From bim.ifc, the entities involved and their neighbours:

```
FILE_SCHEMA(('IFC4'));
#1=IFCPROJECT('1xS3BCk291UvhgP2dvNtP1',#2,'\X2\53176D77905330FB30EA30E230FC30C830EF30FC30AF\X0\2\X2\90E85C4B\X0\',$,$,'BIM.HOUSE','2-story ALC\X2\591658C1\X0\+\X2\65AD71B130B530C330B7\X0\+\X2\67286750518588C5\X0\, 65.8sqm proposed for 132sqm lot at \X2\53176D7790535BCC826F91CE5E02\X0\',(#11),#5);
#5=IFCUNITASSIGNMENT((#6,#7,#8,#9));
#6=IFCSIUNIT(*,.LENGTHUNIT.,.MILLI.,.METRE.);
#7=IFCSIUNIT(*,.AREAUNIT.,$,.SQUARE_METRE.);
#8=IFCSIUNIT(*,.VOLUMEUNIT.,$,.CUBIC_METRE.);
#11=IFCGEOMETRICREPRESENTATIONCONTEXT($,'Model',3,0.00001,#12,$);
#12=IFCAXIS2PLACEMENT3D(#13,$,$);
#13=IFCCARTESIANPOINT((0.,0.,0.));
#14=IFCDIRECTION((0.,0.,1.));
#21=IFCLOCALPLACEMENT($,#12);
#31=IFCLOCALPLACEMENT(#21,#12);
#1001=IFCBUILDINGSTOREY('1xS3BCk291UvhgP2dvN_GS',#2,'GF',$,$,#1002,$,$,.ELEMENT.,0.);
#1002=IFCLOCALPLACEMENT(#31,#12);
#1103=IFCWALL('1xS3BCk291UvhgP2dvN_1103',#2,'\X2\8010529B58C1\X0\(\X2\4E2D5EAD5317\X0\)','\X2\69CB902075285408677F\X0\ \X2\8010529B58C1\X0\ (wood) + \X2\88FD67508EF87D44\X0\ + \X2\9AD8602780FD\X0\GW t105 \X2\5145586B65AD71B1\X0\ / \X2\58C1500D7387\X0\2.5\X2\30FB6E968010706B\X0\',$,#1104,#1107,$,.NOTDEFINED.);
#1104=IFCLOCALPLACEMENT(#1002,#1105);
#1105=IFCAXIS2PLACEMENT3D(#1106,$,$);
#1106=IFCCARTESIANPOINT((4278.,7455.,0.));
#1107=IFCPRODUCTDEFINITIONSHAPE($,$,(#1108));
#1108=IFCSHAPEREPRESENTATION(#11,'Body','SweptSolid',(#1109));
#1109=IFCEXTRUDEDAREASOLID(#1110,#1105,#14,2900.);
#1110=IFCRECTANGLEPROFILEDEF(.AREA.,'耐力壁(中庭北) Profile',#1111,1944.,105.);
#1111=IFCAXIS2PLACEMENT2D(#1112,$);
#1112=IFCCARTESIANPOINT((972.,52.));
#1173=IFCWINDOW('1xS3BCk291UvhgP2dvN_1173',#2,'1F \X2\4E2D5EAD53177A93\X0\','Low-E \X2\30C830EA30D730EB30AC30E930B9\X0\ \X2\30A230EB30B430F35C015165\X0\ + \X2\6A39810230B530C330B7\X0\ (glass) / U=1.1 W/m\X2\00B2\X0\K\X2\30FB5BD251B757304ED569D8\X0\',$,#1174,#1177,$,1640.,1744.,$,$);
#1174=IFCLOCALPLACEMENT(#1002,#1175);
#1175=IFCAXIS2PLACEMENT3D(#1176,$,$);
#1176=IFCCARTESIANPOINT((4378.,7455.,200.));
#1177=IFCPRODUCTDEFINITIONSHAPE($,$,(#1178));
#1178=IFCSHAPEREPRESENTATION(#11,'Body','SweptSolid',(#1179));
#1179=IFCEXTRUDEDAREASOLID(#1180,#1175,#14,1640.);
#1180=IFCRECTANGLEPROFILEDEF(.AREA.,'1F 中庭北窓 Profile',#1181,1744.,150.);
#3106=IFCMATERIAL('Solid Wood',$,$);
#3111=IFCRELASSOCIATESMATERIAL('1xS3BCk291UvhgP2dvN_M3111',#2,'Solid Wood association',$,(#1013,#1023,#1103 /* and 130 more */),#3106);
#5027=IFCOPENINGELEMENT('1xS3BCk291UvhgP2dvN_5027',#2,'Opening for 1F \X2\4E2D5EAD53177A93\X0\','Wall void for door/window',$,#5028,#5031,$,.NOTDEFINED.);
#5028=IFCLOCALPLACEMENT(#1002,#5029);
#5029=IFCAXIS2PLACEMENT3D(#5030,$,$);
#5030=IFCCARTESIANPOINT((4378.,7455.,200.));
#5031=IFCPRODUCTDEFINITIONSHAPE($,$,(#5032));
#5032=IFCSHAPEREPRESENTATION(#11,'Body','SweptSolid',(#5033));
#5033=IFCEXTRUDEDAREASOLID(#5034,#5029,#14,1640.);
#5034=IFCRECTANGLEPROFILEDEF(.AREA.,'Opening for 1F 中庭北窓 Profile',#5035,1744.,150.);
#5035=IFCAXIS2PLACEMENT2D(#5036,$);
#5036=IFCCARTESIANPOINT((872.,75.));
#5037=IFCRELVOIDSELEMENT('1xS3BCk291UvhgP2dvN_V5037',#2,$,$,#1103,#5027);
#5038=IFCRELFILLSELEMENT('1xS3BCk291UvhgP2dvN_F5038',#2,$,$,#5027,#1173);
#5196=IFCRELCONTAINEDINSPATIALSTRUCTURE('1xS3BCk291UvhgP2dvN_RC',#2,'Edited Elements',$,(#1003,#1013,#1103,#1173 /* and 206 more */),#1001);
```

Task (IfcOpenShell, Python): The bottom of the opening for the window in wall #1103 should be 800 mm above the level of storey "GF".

```python
import numpy as np
import ifcopenshell
import ifcopenshell.api.geometry
import ifcopenshell.geom
import ifcopenshell.util.element
import ifcopenshell.util.placement
import ifcopenshell.util.shape
import ifcopenshell.util.unit

model = ifcopenshell.open("bim.ifc")
unit_scale = ifcopenshell.util.unit.calculate_unit_scale(model)

window = model.by_guid("1xS3BCk291UvhgP2dvN_1173")
opening = window.FillsVoids[0].RelatingOpeningElement
storey = ifcopenshell.util.element.get_container(window, ifc_class="IfcBuildingStorey")
level = ifcopenshell.util.placement.get_local_placement(storey.ObjectPlacement)[2, 3]

# The opening's origin need not be at the sill, so measure its lowest point.
shape = ifcopenshell.geom.create_shape(ifcopenshell.geom.settings(), opening)
bottom = ifcopenshell.util.shape.get_shape_bottom_elevation(shape, shape.geometry) / unit_scale
dz = level + 0.8 / unit_scale - bottom

shift = np.array([0.0, 0.0, dz])
# The window is not placed relative to its opening, so move both.
for product in (opening, window):
    matrix = ifcopenshell.util.placement.get_local_placement(product.ObjectPlacement)
    matrix[:3, 3] += shift
    ifcopenshell.api.geometry.edit_object_placement(model, product=product, matrix=matrix, is_si=False)

print(f"moved by {dz * unit_scale:+.3f} m")

model.write("bim-out.ifc")
```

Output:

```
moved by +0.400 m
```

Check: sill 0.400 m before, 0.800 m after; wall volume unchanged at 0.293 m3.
